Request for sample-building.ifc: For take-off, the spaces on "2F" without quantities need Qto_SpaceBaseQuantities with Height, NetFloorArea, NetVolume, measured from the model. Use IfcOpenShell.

First a look at what the model holds.

```python
import ifcopenshell
import ifcopenshell.util.element
import ifcopenshell.util.unit

model = ifcopenshell.open("sample-building.ifc")
print(model.schema)
for unit_type in ("LENGTHUNIT", "AREAUNIT", "VOLUMEUNIT"):
    print(unit_type, ifcopenshell.util.unit.calculate_unit_scale(model, unit_type))
storey = next(s for s in model.by_type("IfcBuildingStorey") if s.Name == "2F")
spaces = [e for e in ifcopenshell.util.element.get_decomposition(storey) if e.is_a("IfcSpace")]
for e in sorted(spaces, key=lambda e: e.id()):
    print(e.id(), e.is_a(), e.Name, list(ifcopenshell.util.element.get_psets(e, qtos_only=True)), sep=" | ")
```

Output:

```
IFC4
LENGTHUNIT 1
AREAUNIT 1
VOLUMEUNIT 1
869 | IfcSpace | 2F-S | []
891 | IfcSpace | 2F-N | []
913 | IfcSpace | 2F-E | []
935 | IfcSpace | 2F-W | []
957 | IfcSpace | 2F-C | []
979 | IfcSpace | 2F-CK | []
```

```python
import ifcopenshell
import ifcopenshell.api.pset
import ifcopenshell.geom
import ifcopenshell.util.element
import ifcopenshell.util.shape
import ifcopenshell.util.unit

model = ifcopenshell.open("sample-building.ifc")
unit_scale = ifcopenshell.util.unit.calculate_unit_scale(model)
area_scale = ifcopenshell.util.unit.calculate_unit_scale(model, "AREAUNIT")
volume_scale = ifcopenshell.util.unit.calculate_unit_scale(model, "VOLUMEUNIT")
settings = ifcopenshell.geom.settings()

storey = next(s for s in model.by_type("IfcBuildingStorey") if s.Name == "2F")
spaces = [e for e in ifcopenshell.util.element.get_decomposition(storey) if e.is_a("IfcSpace")]

for e in sorted(spaces, key=lambda e: e.id()):
    if ifcopenshell.util.element.get_psets(e, qtos_only=True, should_inherit=False):
        continue
    # Geometry comes back in metres, in the element's own axes.
    shape = ifcopenshell.geom.create_shape(settings, e)
    values = {
        "Height": ifcopenshell.util.shape.get_z(shape.geometry) / unit_scale,
        "NetFloorArea": ifcopenshell.util.shape.get_footprint_area(shape.geometry) / area_scale,
        "NetVolume": ifcopenshell.util.shape.get_volume(shape.geometry) / volume_scale,
    }
    qto = ifcopenshell.api.pset.add_qto(model, product=e, name="Qto_SpaceBaseQuantities")
    ifcopenshell.api.pset.edit_qto(model, qto=qto, properties=values)
    print(e.id(), {k: round(v, 3) for k, v in values.items()})

model.write("sample-building_v2.ifc")
```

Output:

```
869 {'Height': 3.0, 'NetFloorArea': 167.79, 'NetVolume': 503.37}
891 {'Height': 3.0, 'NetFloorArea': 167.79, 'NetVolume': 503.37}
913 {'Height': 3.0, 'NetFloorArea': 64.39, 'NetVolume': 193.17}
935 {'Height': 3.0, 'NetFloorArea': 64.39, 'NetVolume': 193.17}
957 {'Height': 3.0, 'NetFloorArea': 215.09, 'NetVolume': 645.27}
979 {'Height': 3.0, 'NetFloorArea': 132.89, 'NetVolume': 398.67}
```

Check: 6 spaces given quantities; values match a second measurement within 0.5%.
